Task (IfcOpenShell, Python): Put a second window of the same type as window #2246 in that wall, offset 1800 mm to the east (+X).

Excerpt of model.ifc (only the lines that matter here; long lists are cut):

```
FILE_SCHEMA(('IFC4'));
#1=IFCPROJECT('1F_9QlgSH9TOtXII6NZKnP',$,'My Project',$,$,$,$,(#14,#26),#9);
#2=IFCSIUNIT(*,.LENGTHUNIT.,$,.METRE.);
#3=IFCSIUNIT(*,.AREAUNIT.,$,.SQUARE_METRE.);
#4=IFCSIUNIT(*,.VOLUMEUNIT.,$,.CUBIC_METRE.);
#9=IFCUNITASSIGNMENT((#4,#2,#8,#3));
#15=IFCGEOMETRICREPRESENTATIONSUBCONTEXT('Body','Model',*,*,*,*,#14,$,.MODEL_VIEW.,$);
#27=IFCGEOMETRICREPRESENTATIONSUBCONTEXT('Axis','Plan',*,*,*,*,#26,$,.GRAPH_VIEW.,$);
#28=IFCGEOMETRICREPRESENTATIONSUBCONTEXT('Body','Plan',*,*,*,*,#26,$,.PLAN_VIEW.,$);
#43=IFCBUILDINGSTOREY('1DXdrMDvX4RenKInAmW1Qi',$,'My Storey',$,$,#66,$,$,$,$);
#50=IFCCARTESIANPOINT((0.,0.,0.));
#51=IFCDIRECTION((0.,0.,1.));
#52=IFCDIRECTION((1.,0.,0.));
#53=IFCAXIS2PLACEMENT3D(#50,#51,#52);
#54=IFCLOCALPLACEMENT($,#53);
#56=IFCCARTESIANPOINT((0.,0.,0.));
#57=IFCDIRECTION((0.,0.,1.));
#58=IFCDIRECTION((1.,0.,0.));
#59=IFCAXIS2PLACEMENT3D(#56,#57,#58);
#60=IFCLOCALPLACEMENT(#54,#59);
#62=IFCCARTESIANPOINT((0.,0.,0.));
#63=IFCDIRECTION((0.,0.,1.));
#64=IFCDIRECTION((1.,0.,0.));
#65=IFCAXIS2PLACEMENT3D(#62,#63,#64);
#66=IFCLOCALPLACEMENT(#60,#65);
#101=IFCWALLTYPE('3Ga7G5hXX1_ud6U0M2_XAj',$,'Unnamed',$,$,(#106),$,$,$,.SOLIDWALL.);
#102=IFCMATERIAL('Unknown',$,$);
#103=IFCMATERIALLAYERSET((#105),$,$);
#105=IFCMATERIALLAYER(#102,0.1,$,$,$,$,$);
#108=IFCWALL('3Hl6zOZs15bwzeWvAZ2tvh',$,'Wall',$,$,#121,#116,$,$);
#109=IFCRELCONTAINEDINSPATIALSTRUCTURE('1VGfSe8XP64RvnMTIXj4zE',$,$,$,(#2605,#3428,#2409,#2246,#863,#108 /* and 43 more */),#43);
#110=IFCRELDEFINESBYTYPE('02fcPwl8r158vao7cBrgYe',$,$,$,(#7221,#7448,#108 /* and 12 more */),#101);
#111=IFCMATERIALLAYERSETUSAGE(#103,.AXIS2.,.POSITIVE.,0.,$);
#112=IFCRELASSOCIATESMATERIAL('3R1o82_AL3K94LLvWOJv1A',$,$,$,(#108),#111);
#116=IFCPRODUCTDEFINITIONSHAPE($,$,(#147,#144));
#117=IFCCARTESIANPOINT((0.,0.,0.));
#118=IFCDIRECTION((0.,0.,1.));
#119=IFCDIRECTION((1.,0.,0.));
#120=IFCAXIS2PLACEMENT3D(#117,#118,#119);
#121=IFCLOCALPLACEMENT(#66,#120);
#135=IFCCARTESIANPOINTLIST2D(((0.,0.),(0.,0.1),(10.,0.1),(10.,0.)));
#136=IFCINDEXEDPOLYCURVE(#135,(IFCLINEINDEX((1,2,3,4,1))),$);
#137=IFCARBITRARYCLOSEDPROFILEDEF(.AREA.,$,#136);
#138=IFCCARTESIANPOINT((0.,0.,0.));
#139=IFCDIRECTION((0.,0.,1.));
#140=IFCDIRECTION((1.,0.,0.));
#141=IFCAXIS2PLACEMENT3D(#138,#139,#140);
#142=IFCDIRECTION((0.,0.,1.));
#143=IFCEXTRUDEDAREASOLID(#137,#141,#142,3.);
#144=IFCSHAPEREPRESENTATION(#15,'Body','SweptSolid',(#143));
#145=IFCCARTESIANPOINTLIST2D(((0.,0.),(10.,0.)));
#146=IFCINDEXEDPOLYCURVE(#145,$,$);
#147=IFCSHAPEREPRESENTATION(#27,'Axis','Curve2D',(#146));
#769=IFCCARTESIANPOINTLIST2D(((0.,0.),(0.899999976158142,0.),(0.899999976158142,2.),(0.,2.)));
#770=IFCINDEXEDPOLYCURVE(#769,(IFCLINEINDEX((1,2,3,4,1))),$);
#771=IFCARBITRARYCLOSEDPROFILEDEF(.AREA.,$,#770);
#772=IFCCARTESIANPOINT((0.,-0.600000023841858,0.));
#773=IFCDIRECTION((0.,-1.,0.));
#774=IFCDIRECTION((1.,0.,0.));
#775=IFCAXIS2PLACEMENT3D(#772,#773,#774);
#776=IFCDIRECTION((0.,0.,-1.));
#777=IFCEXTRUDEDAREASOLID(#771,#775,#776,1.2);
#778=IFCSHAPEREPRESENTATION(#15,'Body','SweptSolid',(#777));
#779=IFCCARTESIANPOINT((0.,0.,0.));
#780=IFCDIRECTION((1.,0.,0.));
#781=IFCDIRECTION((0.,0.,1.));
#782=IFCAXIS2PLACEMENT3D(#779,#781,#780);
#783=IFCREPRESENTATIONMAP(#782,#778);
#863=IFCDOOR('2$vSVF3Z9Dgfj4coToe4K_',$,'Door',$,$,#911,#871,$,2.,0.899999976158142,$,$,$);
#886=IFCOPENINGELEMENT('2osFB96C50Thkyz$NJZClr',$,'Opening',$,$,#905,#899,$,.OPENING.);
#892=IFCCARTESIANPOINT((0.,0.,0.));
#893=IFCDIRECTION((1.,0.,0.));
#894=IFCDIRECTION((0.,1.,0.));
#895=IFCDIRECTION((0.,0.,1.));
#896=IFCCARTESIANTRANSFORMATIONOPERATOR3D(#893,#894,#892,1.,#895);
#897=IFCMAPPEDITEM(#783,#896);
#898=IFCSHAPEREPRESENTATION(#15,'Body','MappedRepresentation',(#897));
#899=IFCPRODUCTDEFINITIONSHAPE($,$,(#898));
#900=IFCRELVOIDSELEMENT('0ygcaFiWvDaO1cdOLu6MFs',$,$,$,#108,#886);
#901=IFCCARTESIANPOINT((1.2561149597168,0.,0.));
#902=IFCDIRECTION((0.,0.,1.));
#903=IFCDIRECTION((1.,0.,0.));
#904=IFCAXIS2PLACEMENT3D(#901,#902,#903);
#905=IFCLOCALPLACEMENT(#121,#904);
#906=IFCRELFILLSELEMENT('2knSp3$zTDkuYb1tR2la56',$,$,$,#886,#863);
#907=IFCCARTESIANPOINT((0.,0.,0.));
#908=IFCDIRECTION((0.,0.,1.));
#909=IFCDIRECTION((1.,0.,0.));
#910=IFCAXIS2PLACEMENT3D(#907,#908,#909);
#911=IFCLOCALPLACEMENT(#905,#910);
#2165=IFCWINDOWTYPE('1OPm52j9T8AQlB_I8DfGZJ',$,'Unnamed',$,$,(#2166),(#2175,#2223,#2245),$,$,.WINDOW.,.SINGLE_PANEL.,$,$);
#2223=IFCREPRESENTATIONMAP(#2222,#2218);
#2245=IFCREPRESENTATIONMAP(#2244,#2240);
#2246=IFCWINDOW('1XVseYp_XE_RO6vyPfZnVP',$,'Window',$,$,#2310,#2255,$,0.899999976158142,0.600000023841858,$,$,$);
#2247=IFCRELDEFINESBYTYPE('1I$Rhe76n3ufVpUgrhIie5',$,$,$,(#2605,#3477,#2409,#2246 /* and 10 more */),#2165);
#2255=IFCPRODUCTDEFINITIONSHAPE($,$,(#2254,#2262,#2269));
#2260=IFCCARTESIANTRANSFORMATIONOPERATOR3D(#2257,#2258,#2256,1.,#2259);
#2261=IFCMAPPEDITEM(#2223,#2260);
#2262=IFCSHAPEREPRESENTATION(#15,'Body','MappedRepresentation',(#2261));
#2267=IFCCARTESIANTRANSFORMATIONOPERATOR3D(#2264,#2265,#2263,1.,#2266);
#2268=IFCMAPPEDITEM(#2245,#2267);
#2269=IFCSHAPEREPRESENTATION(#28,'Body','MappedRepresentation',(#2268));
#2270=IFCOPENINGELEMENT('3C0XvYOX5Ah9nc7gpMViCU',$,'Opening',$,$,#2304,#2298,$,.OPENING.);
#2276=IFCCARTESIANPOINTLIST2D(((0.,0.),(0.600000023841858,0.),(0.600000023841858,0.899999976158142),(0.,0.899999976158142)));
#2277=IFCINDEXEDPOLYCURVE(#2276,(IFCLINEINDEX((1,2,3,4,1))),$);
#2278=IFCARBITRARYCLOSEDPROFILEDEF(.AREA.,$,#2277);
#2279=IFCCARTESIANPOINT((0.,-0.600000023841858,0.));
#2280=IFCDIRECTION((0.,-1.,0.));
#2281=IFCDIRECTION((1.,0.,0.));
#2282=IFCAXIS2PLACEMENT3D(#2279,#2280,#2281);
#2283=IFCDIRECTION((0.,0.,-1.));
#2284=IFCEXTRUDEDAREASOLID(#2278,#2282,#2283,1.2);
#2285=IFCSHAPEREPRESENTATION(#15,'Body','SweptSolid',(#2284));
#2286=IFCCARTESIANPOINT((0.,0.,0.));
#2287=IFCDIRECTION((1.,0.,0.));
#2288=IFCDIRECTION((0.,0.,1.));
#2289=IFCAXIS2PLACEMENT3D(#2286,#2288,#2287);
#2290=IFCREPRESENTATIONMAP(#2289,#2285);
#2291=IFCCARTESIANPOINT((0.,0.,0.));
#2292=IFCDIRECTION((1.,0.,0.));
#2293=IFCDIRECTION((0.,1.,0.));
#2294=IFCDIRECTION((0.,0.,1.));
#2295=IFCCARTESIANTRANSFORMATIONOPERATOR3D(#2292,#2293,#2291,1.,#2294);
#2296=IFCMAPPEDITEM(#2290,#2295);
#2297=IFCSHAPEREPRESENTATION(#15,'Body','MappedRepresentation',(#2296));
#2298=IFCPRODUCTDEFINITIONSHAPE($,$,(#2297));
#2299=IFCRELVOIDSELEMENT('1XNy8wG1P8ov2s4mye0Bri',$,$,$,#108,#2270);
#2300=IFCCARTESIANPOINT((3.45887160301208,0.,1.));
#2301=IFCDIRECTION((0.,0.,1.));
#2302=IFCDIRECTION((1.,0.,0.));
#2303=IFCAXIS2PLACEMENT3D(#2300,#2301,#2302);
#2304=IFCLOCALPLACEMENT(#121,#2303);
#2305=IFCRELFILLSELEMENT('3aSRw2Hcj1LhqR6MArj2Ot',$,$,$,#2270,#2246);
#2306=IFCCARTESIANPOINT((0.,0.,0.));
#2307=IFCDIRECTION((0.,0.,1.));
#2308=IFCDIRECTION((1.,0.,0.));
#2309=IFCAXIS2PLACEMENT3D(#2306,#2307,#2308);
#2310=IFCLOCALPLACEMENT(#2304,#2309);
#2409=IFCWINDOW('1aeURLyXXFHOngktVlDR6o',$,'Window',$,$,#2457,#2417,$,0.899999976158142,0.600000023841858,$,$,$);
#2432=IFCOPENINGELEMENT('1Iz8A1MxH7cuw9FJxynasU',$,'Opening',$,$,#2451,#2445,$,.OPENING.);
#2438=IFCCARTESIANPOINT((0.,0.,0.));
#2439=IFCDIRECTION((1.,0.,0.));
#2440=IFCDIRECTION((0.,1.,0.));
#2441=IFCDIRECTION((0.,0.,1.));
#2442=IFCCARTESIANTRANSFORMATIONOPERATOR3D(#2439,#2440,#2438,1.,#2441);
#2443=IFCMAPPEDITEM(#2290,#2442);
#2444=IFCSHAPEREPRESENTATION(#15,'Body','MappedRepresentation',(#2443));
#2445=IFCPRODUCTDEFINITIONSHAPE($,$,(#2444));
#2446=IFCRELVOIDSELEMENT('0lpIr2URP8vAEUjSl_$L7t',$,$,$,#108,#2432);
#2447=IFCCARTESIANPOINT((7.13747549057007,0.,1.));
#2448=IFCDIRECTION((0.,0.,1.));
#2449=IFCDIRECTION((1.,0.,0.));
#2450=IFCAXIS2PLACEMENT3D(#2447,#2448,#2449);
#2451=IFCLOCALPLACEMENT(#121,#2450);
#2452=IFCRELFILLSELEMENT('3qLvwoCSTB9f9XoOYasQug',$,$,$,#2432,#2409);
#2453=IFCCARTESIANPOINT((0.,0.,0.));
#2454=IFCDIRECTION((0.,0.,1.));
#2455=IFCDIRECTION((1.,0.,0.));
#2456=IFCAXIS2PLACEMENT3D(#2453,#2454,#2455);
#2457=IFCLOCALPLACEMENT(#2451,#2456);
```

```python
import ifcopenshell
import ifcopenshell.api.feature
import ifcopenshell.api.geometry
import ifcopenshell.api.root
import ifcopenshell.geom
import ifcopenshell.util.element
import ifcopenshell.util.placement
import ifcopenshell.util.shape

model = ifcopenshell.open("model.ifc")
settings = ifcopenshell.geom.settings()


def volume(element):
    """Net volume in cubic metres, openings subtracted."""
    shape = ifcopenshell.geom.create_shape(settings, element)
    return ifcopenshell.util.shape.get_volume(shape.geometry)


window = model.by_guid("1XVseYp_XE_RO6vyPfZnVP")
opening = window.FillsVoids[0].RelatingOpeningElement
wall = opening.VoidsElements[0].RelatingBuildingElement
before = volume(wall)
shift = ifcopenshell.util.placement.get_local_placement(wall.ObjectPlacement)[:3, 0] * 1.8

# copy_class copies the void relationship, type, container and properties, but no geometry.
new_opening = ifcopenshell.api.root.copy_class(model, product=opening)
new_opening.Representation = ifcopenshell.util.element.copy_deep(
    model, opening.Representation, exclude=["IfcGeometricRepresentationContext", "IfcRepresentationMap"]
)
new_window = ifcopenshell.api.root.copy_class(model, product=window)
new_window.Representation = ifcopenshell.util.element.copy_deep(
    model, window.Representation, exclude=["IfcGeometricRepresentationContext", "IfcRepresentationMap"]
)
ifcopenshell.api.feature.add_filling(model, opening=new_opening, element=new_window)

for old, new in ((opening, new_opening), (window, new_window)):
    matrix = ifcopenshell.util.placement.get_local_placement(old.ObjectPlacement)
    matrix[:3, 3] += shift
    ifcopenshell.api.geometry.edit_object_placement(model, product=new, matrix=matrix, is_si=False)

after = volume(wall)

print(f"wall volume {before:.3f} -> {after:.3f} m3")

model.write("model_updated.ifc")
```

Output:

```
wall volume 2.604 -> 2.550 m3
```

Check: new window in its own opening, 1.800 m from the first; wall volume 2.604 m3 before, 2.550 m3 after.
